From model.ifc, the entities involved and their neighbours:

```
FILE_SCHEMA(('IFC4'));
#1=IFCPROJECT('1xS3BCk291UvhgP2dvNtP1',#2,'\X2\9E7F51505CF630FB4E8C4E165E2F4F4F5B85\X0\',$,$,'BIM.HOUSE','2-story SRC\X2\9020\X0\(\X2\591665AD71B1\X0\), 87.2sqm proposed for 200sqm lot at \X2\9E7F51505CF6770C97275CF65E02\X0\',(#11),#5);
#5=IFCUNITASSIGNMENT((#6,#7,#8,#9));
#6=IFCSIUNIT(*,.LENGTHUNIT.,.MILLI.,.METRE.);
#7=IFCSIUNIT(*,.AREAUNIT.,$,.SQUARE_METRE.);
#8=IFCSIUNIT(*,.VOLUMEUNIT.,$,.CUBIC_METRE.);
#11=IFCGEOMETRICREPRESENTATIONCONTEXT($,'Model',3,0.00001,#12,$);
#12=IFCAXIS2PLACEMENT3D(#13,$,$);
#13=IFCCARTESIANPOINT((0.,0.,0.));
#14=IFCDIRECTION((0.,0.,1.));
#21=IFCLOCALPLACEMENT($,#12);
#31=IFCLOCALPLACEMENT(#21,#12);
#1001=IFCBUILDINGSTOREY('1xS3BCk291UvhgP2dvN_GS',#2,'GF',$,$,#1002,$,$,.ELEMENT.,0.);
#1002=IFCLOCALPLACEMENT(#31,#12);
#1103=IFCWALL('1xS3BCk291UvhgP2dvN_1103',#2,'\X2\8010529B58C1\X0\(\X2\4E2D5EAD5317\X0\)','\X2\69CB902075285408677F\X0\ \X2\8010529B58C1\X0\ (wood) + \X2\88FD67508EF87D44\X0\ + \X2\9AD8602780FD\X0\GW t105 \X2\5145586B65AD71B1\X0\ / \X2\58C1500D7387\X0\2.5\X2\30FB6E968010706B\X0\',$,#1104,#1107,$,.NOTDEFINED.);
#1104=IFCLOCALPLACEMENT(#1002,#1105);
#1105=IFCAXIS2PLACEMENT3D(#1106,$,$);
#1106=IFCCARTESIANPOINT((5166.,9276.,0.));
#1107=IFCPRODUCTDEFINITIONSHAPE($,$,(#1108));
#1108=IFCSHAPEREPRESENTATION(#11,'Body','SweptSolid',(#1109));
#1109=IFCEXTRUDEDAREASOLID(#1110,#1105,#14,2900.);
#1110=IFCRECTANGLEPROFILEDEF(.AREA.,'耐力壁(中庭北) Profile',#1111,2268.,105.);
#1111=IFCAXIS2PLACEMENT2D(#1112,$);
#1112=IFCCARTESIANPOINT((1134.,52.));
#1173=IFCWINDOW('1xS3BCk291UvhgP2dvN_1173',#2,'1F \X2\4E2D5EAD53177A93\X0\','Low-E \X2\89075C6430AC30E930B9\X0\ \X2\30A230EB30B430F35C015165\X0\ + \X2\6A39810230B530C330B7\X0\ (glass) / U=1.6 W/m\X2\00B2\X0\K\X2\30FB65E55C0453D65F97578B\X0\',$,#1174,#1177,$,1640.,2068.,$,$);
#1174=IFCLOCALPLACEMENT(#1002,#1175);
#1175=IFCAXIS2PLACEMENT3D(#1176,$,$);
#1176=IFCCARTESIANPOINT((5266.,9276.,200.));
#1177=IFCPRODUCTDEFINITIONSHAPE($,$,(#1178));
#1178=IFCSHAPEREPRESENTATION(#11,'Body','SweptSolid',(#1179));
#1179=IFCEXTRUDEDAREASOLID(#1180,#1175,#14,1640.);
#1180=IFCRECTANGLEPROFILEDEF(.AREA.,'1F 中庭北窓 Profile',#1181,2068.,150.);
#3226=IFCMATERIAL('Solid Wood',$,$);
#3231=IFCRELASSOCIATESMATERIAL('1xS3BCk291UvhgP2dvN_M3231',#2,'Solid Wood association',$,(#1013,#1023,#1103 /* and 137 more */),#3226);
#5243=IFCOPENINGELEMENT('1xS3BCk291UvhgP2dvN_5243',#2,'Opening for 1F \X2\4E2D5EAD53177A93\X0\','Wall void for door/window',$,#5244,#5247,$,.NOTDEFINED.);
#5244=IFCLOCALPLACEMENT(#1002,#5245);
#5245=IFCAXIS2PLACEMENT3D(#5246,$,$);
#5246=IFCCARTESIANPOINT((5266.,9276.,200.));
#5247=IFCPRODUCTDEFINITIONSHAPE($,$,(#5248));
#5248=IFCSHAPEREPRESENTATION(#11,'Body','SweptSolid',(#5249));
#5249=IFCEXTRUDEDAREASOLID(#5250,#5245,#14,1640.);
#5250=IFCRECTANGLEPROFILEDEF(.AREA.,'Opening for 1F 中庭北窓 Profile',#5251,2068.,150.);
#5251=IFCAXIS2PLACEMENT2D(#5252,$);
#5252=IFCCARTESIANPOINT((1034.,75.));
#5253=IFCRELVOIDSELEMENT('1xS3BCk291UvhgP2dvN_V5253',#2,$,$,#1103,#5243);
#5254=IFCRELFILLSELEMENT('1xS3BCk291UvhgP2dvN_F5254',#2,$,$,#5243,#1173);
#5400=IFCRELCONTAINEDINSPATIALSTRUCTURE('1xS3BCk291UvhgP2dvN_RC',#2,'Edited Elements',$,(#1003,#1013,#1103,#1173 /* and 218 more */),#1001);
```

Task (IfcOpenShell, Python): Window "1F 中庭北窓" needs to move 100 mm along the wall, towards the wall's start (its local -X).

```python
import ifcopenshell
import ifcopenshell.api.geometry
import ifcopenshell.util.placement
import ifcopenshell.util.unit

model = ifcopenshell.open("model.ifc")
unit_scale = ifcopenshell.util.unit.calculate_unit_scale(model)

window = model.by_guid("1xS3BCk291UvhgP2dvN_1173")
opening = window.FillsVoids[0].RelatingOpeningElement
wall = opening.VoidsElements[0].RelatingBuildingElement

wall_matrix = ifcopenshell.util.placement.get_local_placement(wall.ObjectPlacement)
shift = wall_matrix[:3, 0] * -0.1 / unit_scale
before = ifcopenshell.util.placement.get_local_placement(window.ObjectPlacement)[:3, 3].copy()

# The window is not placed relative to its opening, so move both.
for product in (opening, window):
    matrix = ifcopenshell.util.placement.get_local_placement(product.ObjectPlacement)
    matrix[:3, 3] += shift
    ifcopenshell.api.geometry.edit_object_placement(model, product=product, matrix=matrix, is_si=False)

after = ifcopenshell.util.placement.get_local_placement(window.ObjectPlacement)[:3, 3]
print("window moved by", (after - before).round(3) + 0.0)

model.write("model_rev.ifc")
```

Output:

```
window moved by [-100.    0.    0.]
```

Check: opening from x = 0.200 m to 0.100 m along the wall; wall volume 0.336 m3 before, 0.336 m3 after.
